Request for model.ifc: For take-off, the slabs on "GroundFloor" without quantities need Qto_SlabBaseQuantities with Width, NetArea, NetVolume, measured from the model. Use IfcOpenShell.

First a look at what the model holds.

```python
import ifcopenshell
import ifcopenshell.util.element
import ifcopenshell.util.unit

model = ifcopenshell.open("model.ifc")
print(model.schema)
for unit_type in ("LENGTHUNIT", "AREAUNIT", "VOLUMEUNIT"):
    print(unit_type, ifcopenshell.util.unit.calculate_unit_scale(model, unit_type))
storey = next(s for s in model.by_type("IfcBuildingStorey") if s.Name == "GroundFloor")
slabs = [e for e in ifcopenshell.util.element.get_decomposition(storey) if e.is_a("IfcSlab")]
for e in sorted(slabs, key=lambda e: e.id()):
    print(e.id(), e.is_a(), e.Name, list(ifcopenshell.util.element.get_psets(e, qtos_only=True)), sep=" | ")
```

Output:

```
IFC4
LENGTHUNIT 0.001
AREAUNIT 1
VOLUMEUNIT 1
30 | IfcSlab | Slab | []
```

```python
import ifcopenshell
import ifcopenshell.api.pset
import ifcopenshell.geom
import ifcopenshell.util.element
import ifcopenshell.util.shape
import ifcopenshell.util.unit

model = ifcopenshell.open("model.ifc")
unit_scale = ifcopenshell.util.unit.calculate_unit_scale(model)
area_scale = ifcopenshell.util.unit.calculate_unit_scale(model, "AREAUNIT")
volume_scale = ifcopenshell.util.unit.calculate_unit_scale(model, "VOLUMEUNIT")
settings = ifcopenshell.geom.settings()

storey = next(s for s in model.by_type("IfcBuildingStorey") if s.Name == "GroundFloor")
slabs = [e for e in ifcopenshell.util.element.get_decomposition(storey) if e.is_a("IfcSlab")]

for e in sorted(slabs, key=lambda e: e.id()):
    if ifcopenshell.util.element.get_psets(e, qtos_only=True, should_inherit=False):
        continue
    # Geometry comes back in metres, in the element's own axes.
    shape = ifcopenshell.geom.create_shape(settings, e)
    values = {
        "Width": ifcopenshell.util.shape.get_z(shape.geometry) / unit_scale,
        "NetArea": ifcopenshell.util.shape.get_footprint_area(shape.geometry) / area_scale,
        "NetVolume": ifcopenshell.util.shape.get_volume(shape.geometry) / volume_scale,
    }
    qto = ifcopenshell.api.pset.add_qto(model, product=e, name="Qto_SlabBaseQuantities")
    ifcopenshell.api.pset.edit_qto(model, qto=qto, properties=values)
    print(e.id(), {k: round(v, 3) for k, v in values.items()})

model.write("model_rev.ifc")
```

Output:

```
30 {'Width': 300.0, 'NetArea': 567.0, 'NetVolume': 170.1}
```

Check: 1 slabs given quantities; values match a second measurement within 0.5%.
